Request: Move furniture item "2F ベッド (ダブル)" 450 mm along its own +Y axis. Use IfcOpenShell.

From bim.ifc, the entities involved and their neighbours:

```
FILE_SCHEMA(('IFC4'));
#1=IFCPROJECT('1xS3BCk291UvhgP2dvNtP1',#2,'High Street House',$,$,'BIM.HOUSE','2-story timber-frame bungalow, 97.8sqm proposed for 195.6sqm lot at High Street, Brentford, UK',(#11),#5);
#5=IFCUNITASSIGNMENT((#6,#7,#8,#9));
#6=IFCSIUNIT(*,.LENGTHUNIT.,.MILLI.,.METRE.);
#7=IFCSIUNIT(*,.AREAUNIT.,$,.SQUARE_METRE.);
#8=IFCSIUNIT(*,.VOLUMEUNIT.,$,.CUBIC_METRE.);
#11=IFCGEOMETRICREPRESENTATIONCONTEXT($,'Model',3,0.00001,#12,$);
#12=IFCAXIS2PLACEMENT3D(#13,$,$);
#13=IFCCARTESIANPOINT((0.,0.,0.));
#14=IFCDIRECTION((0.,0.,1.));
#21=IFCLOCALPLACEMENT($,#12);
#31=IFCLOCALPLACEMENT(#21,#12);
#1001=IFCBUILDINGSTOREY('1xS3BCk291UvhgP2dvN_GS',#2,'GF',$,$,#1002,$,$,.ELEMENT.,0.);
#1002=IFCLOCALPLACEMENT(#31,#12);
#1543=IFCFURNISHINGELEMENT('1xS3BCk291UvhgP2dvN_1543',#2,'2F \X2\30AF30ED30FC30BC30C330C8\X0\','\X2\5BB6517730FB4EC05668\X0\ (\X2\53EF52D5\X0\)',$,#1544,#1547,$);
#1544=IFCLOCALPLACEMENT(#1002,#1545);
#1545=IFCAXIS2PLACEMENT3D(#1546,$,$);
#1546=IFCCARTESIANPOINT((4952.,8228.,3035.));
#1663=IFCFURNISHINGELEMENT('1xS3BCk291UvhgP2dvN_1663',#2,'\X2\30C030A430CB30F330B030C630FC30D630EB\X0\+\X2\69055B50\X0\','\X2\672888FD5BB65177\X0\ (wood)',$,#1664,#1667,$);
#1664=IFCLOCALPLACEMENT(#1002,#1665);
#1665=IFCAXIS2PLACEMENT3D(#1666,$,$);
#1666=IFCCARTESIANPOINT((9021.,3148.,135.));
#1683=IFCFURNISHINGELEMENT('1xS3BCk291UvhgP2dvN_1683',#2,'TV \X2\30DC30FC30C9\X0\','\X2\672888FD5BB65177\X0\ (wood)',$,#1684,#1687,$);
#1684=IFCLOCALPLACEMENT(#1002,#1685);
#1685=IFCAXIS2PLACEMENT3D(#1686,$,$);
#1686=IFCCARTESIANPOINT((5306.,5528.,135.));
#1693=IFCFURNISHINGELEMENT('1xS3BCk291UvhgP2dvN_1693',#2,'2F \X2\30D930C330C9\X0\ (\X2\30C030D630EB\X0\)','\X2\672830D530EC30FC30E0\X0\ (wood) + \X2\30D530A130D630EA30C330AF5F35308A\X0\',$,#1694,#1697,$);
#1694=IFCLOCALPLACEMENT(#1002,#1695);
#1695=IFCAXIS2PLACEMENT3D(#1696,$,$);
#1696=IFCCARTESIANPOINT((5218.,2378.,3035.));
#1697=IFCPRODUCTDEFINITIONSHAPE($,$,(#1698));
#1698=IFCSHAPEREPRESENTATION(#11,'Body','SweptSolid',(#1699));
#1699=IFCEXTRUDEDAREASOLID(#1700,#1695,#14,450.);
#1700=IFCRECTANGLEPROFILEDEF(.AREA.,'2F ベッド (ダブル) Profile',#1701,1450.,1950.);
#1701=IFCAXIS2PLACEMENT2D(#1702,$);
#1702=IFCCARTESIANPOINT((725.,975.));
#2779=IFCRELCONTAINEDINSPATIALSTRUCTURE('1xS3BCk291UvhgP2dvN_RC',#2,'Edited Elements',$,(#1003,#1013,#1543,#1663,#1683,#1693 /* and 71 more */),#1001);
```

```python
import ifcopenshell
import ifcopenshell.api.geometry
import ifcopenshell.util.placement

model = ifcopenshell.open("bim.ifc")

item = model.by_guid("1xS3BCk291UvhgP2dvN_1693")
matrix = ifcopenshell.util.placement.get_local_placement(item.ObjectPlacement)
matrix[:3, 3] += matrix[:3, 1] * 450.0
ifcopenshell.api.geometry.edit_object_placement(model, product=item, matrix=matrix, is_si=False)

print(ifcopenshell.util.placement.get_local_placement(item.ObjectPlacement).round(3) + 0.0)

model.write("bim-out.ifc")
```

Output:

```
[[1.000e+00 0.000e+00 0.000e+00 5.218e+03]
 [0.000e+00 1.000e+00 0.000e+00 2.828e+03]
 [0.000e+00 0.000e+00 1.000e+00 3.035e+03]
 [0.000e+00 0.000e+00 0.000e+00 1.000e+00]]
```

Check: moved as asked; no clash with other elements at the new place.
